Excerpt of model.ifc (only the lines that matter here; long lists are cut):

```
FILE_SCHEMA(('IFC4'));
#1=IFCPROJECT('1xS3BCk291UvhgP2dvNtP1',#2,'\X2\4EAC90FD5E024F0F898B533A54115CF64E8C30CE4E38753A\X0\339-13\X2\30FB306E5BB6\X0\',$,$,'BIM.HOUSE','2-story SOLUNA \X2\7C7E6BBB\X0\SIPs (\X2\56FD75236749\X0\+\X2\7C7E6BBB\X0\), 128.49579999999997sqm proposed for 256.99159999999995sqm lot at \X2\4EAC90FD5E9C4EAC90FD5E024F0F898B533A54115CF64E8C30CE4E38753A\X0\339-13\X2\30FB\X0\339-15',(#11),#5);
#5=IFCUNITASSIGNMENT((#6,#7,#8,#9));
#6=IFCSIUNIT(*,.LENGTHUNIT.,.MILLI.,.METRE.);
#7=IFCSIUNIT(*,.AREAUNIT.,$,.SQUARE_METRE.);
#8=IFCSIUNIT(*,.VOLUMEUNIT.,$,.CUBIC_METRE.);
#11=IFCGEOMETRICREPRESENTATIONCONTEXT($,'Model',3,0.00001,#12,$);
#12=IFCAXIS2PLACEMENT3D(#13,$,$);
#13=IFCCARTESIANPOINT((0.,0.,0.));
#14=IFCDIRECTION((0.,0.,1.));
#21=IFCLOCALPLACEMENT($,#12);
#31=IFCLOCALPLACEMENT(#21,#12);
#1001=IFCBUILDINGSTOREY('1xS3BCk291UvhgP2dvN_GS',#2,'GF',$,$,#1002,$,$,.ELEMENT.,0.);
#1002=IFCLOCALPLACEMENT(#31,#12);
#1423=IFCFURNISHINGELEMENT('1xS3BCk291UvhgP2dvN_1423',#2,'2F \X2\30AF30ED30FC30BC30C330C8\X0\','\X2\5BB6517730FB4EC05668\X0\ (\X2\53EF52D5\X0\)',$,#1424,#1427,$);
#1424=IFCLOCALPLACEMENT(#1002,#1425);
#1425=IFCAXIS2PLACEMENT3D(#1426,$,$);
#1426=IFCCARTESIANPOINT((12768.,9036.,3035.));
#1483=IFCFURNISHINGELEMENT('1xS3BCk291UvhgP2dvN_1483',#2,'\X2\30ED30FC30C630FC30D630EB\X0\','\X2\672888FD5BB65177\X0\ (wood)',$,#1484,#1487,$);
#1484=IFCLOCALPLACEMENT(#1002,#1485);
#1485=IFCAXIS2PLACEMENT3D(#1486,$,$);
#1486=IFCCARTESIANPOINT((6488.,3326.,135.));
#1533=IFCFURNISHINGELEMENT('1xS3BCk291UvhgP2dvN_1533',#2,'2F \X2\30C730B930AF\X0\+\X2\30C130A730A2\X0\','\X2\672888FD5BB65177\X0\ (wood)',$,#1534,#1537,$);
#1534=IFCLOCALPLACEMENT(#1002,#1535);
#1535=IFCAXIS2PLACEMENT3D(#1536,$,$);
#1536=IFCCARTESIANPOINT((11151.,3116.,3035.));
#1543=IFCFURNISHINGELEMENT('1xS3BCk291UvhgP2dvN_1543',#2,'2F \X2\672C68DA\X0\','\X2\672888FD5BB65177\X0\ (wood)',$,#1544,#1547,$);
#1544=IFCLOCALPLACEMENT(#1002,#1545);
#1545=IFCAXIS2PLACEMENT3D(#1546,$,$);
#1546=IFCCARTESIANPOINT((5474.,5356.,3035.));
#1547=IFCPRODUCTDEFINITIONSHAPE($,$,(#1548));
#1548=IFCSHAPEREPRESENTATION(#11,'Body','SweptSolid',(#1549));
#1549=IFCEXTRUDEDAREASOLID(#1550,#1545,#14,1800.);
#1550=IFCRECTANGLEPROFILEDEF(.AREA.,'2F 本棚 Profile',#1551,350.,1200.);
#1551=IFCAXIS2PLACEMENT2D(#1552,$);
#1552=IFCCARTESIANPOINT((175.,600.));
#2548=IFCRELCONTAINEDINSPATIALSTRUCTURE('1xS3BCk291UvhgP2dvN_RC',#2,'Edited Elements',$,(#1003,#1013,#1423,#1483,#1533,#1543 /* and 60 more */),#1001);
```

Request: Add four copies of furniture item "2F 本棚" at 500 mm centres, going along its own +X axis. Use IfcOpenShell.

```python
import ifcopenshell
import ifcopenshell.api.geometry
import ifcopenshell.api.root
import ifcopenshell.util.element
import ifcopenshell.util.placement
import ifcopenshell.util.unit

model = ifcopenshell.open("model.ifc")
unit_scale = ifcopenshell.util.unit.calculate_unit_scale(model)


def reuse_history(source, copy):
    """copy_class also copies each property set's owner history, people and application; keep the originals."""
    for rel in copy.IsDefinedBy:
        if rel.is_a("IfcRelDefinesByProperties") and (history := rel.RelatingPropertyDefinition.OwnerHistory):
            rel.RelatingPropertyDefinition.OwnerHistory = source.OwnerHistory
            ifcopenshell.util.element.remove_deep2(model, history)


source = model.by_id(1543)
base = ifcopenshell.util.placement.get_local_placement(source.ObjectPlacement)
step = base[:3, 0] * 0.5 / unit_scale

for i in range(1, 5):
    copy = ifcopenshell.api.root.copy_class(model, product=source)
    copy.Representation = ifcopenshell.util.element.copy_deep(
        model, source.Representation, exclude=["IfcGeometricRepresentationContext", "IfcRepresentationMap"]
    )
    reuse_history(source, copy)
    matrix = base.copy()
    matrix[:3, 3] += i * step
    print("added at", matrix[:3, 3].round(3) + 0.0)
    ifcopenshell.api.geometry.edit_object_placement(model, product=copy, matrix=matrix, is_si=False)

model.write("model_updated.ifc")
```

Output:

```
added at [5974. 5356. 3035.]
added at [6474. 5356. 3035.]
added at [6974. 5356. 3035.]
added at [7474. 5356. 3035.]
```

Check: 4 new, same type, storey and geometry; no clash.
